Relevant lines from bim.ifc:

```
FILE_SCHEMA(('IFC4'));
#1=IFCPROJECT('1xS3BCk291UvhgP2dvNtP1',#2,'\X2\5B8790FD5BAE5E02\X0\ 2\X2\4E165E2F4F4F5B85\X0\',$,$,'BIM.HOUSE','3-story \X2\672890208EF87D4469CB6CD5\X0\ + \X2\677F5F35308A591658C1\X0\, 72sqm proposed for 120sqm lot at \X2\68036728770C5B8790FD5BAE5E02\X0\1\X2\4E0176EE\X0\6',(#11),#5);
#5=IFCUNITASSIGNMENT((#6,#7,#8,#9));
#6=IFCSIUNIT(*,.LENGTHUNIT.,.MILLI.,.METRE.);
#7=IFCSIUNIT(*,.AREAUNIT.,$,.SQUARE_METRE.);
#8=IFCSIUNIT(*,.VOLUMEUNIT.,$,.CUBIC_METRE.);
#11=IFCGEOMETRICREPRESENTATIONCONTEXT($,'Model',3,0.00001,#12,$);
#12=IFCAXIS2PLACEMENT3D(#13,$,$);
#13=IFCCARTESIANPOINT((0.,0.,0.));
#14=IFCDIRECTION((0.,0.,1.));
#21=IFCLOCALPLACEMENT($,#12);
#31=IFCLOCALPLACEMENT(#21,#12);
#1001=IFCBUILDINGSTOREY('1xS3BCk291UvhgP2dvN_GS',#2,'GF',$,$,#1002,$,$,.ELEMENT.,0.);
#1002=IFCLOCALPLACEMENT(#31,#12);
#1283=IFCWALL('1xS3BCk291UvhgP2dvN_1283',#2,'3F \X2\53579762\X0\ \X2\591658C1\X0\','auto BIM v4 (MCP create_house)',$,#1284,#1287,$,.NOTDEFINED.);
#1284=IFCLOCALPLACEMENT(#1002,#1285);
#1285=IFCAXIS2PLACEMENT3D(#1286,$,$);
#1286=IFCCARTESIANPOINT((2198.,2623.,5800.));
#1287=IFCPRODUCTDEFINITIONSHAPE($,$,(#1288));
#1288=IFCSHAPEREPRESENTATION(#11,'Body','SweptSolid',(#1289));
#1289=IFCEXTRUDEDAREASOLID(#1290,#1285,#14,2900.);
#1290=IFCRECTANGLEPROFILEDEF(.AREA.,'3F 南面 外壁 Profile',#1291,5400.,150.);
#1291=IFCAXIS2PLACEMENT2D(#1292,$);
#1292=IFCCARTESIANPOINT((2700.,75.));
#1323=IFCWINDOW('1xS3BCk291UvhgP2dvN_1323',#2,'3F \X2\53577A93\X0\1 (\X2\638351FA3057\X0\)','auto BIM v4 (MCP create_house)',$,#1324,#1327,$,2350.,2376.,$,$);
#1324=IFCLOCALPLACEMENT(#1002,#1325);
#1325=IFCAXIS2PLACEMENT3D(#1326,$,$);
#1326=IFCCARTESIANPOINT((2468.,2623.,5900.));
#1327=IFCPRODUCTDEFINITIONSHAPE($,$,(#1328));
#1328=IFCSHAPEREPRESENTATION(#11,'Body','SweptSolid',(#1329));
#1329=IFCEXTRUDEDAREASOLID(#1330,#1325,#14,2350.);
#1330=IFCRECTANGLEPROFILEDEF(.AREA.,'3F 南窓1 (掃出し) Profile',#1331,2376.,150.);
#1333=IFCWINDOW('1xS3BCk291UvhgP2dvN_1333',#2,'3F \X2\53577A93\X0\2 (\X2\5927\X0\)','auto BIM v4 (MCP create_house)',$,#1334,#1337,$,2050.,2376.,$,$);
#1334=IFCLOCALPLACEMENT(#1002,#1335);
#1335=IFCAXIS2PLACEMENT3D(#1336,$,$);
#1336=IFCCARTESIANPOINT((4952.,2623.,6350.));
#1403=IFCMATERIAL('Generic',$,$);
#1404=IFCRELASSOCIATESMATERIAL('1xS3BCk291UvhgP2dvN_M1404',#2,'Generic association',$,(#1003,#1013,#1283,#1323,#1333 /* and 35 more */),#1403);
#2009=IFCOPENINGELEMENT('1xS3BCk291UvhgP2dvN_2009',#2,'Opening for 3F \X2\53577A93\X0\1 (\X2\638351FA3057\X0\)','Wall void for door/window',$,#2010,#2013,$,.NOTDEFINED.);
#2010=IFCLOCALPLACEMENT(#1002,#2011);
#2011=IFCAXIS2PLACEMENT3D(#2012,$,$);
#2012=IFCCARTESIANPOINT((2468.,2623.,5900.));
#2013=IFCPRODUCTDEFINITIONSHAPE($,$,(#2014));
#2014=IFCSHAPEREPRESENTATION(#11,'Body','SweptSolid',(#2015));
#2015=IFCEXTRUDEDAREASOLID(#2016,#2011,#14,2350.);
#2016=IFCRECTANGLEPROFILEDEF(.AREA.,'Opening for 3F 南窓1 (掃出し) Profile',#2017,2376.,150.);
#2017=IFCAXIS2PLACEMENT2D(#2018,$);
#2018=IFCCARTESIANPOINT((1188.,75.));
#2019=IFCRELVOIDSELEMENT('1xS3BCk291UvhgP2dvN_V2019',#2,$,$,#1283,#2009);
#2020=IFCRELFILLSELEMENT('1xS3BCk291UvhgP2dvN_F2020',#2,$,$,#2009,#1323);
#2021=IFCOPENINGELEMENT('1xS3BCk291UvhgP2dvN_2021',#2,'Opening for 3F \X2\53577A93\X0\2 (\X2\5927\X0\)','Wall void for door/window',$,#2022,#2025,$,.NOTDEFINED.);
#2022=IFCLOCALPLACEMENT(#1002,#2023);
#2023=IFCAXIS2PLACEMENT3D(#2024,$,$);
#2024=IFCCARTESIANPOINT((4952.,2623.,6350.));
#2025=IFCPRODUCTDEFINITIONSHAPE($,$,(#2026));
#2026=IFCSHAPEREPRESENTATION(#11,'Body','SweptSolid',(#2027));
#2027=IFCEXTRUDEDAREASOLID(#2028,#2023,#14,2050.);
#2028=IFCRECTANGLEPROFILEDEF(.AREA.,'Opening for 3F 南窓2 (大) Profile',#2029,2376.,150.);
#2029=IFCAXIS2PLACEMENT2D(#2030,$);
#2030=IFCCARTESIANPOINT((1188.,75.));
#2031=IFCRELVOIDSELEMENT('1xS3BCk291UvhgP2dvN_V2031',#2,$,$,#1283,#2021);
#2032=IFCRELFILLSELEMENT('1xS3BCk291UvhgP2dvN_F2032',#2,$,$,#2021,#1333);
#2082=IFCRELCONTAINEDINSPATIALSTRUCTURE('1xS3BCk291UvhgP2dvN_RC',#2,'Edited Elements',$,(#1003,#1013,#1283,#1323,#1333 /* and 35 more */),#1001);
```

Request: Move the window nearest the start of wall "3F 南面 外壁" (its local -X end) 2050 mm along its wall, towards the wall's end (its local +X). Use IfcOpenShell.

```python
import ifcopenshell
import ifcopenshell.api.geometry
import ifcopenshell.util.placement
import ifcopenshell.util.unit

model = ifcopenshell.open("bim.ifc")
unit_scale = ifcopenshell.util.unit.calculate_unit_scale(model)

window = model.by_guid("1xS3BCk291UvhgP2dvN_1323")
opening = window.FillsVoids[0].RelatingOpeningElement
wall = opening.VoidsElements[0].RelatingBuildingElement

wall_matrix = ifcopenshell.util.placement.get_local_placement(wall.ObjectPlacement)
shift = wall_matrix[:3, 0] * 2.05 / unit_scale
before = ifcopenshell.util.placement.get_local_placement(window.ObjectPlacement)[:3, 3].copy()

# The window is not placed relative to its opening, so move both.
for product in (opening, window):
    matrix = ifcopenshell.util.placement.get_local_placement(product.ObjectPlacement)
    matrix[:3, 3] += shift
    ifcopenshell.api.geometry.edit_object_placement(model, product=product, matrix=matrix, is_si=False)

after = ifcopenshell.util.placement.get_local_placement(window.ObjectPlacement)[:3, 3]
print("window moved by", (after - before).round(3) + 0.0)

model.write("bim_updated.ifc")
```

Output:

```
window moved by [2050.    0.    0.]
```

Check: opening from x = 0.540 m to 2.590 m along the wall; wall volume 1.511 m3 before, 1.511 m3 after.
